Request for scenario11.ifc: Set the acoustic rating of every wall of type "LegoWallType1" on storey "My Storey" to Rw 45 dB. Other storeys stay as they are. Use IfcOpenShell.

First a look at what the model holds.

```python
import ifcopenshell
import ifcopenshell.util.element

model = ifcopenshell.open("scenario11.ifc")
print(model.schema)
storey = next(s for s in model.by_type("IfcBuildingStorey") if s.Name == "My Storey")
walls = [e for e in ifcopenshell.util.element.get_decomposition(storey) if e.is_a("IfcWall")]
seen = {}
for e in walls:
    element_type = ifcopenshell.util.element.get_type(e)
    key = (element_type.Name if element_type != e and element_type else None, ifcopenshell.util.element.get_pset(e, "Pset_WallCommon", "AcousticRating"))
    seen[key] = seen.get(key, 0) + 1
for (name, value), count in sorted(seen.items(), key=str):
    print(count, "x", name, "|", value)
```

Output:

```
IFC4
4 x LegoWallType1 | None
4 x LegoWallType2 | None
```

```python
import ifcopenshell
import ifcopenshell.api.pset
import ifcopenshell.util.element

model = ifcopenshell.open("scenario11.ifc")

storey = next(s for s in model.by_type("IfcBuildingStorey") if s.Name == "My Storey")
walls = [e for e in ifcopenshell.util.element.get_decomposition(storey) if e.is_a("IfcWall")]

count = 0
for e in walls:
    element_type = ifcopenshell.util.element.get_type(e)
    if element_type in (None, e) or element_type.Name != "LegoWallType1":
        continue
    # add_pset returns the element's existing set when there is one.
    pset = ifcopenshell.api.pset.add_pset(model, product=e, name="Pset_WallCommon")
    ifcopenshell.api.pset.edit_pset(model, pset=pset, properties={"AcousticRating": "Rw 45 dB"})
    count += 1

print(count, "walls updated")

model.write("scenario11_v2.ifc")
```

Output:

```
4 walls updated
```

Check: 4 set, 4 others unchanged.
